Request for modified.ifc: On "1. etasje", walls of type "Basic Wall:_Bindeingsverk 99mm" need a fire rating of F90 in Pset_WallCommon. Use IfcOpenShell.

First a look at what the model holds.

```python
import ifcopenshell
import ifcopenshell.util.element

model = ifcopenshell.open("modified.ifc")
print(model.schema)
storey = next(s for s in model.by_type("IfcBuildingStorey") if s.Name == "1. etasje")
walls = [e for e in ifcopenshell.util.element.get_decomposition(storey) if e.is_a("IfcWall")]
seen = {}
for e in walls:
    element_type = ifcopenshell.util.element.get_type(e)
    key = (element_type.Name if element_type != e and element_type else None, ifcopenshell.util.element.get_pset(e, "Pset_WallCommon", "FireRating"))
    seen[key] = seen.get(key, 0) + 1
for (name, value), count in sorted(seen.items(), key=str):
    print(count, "x", name, "|", value)
```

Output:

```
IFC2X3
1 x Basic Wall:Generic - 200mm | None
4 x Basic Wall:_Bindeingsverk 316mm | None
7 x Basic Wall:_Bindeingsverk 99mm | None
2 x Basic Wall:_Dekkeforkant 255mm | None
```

```python
import ifcopenshell
import ifcopenshell.api.pset
import ifcopenshell.util.element

model = ifcopenshell.open("modified.ifc")

storey = next(s for s in model.by_type("IfcBuildingStorey") if s.Name == "1. etasje")
walls = [e for e in ifcopenshell.util.element.get_decomposition(storey) if e.is_a("IfcWall")]

count = 0
for e in walls:
    element_type = ifcopenshell.util.element.get_type(e)
    if element_type in (None, e) or element_type.Name != "Basic Wall:_Bindeingsverk 99mm":
        continue
    # add_pset returns the element's existing set when there is one.
    pset = ifcopenshell.api.pset.add_pset(model, product=e, name="Pset_WallCommon")
    ifcopenshell.api.pset.edit_pset(model, pset=pset, properties={"FireRating": "F90"})
    count += 1

print(count, "walls updated")

model.write("modified_rev.ifc")
```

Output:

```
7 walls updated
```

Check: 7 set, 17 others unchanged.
